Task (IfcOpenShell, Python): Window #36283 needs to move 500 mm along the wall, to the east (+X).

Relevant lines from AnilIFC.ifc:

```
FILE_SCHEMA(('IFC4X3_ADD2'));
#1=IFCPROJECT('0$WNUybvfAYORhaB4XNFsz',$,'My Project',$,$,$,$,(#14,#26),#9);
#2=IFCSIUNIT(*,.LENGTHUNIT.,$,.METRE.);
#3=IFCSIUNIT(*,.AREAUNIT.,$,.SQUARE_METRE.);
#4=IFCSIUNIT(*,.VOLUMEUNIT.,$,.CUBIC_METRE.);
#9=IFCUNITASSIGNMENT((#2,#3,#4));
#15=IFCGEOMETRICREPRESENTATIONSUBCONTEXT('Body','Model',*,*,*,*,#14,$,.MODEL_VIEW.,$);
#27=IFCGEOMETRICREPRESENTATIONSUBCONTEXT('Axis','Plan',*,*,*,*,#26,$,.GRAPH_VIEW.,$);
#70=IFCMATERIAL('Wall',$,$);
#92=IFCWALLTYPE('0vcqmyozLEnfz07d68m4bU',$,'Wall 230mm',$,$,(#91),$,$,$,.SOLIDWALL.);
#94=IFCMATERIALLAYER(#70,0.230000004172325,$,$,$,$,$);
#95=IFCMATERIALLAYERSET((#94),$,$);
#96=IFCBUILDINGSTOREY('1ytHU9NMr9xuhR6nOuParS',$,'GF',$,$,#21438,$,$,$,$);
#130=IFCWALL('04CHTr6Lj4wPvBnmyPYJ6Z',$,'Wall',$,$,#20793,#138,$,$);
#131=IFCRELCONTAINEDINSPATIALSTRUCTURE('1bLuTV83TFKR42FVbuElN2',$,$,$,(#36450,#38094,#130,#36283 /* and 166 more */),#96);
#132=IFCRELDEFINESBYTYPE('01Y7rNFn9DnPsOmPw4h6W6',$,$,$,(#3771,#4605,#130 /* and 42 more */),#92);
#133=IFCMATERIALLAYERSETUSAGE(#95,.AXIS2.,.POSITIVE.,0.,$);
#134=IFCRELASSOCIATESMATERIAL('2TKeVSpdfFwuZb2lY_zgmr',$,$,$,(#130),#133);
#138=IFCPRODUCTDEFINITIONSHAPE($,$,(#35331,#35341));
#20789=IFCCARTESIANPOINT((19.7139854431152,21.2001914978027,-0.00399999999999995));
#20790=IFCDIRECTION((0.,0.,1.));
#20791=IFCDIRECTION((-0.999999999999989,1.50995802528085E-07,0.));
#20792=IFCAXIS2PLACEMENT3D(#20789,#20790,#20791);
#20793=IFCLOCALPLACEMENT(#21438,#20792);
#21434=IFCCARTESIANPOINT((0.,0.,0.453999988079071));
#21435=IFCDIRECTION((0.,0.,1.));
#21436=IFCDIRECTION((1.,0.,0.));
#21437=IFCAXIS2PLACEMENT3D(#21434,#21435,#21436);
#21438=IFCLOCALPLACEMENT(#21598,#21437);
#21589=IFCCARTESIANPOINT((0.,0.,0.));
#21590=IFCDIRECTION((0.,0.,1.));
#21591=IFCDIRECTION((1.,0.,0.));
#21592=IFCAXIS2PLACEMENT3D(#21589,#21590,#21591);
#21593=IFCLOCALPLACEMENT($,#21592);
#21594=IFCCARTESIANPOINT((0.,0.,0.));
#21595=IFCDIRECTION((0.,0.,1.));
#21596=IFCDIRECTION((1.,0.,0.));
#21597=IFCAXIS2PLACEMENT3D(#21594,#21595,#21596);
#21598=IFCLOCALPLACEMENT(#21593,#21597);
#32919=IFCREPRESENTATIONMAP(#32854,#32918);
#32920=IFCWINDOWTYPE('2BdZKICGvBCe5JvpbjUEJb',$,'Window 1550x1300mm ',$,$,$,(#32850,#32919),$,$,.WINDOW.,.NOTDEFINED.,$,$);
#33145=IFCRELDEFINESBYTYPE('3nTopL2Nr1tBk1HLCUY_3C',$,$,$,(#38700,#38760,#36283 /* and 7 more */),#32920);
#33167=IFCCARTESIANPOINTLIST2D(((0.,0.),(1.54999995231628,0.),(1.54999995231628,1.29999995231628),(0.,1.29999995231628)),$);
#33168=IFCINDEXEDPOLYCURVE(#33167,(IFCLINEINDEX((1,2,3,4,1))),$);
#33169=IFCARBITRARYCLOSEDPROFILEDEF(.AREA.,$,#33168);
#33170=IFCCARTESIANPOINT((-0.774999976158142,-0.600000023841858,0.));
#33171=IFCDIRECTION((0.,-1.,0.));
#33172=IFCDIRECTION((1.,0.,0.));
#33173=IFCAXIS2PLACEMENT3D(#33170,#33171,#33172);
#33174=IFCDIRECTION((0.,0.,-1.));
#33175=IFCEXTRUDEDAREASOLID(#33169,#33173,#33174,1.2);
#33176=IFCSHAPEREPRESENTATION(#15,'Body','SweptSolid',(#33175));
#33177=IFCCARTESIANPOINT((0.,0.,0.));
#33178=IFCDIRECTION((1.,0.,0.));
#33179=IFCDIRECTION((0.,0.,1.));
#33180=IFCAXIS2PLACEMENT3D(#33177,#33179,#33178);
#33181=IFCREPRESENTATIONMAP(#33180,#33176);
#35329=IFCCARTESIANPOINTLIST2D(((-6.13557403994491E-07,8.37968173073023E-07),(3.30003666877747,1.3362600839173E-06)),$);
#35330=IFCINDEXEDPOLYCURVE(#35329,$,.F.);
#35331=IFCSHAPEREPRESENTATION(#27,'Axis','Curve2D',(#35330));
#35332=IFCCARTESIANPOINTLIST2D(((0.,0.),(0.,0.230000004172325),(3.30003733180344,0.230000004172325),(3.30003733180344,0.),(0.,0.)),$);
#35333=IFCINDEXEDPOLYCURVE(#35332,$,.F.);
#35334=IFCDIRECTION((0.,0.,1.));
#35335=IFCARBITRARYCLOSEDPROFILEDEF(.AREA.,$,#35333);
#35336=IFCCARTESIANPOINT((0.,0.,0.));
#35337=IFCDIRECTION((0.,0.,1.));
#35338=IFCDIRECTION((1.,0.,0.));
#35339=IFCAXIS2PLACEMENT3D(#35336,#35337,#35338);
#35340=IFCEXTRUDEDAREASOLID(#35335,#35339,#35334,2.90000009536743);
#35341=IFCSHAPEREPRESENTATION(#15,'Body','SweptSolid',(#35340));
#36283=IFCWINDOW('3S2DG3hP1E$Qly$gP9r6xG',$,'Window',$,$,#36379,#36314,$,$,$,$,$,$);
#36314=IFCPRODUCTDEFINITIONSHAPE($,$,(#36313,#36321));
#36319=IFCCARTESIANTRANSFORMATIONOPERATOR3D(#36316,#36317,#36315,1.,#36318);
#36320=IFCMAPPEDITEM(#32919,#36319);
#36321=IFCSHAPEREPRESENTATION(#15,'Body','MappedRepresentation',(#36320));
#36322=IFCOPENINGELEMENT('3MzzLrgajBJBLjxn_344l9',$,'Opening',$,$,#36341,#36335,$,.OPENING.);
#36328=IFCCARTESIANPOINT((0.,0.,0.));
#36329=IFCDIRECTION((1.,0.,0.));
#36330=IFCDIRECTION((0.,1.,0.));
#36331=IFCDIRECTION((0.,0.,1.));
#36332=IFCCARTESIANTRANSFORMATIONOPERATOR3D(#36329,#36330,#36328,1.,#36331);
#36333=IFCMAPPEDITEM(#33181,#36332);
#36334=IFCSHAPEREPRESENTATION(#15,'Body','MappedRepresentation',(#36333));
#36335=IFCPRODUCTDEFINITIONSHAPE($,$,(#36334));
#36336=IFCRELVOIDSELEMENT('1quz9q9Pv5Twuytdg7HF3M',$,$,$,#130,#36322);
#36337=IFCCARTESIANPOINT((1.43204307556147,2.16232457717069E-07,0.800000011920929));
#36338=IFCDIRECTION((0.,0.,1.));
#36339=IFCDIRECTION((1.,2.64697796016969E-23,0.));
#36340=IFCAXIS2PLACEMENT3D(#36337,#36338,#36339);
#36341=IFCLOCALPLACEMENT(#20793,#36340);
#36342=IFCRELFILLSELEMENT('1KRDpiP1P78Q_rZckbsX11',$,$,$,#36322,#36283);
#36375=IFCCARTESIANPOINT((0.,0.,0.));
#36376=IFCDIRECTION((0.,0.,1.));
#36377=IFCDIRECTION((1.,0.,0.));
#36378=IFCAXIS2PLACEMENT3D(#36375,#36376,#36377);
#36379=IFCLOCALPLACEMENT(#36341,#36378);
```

```python
import ifcopenshell
import ifcopenshell.api.geometry
import ifcopenshell.util.placement

model = ifcopenshell.open("AnilIFC.ifc")

window = model.by_guid("3S2DG3hP1E$Qly$gP9r6xG")
opening = window.FillsVoids[0].RelatingOpeningElement
wall = opening.VoidsElements[0].RelatingBuildingElement

wall_matrix = ifcopenshell.util.placement.get_local_placement(wall.ObjectPlacement)
shift = wall_matrix[:3, 0] * -0.5
before = ifcopenshell.util.placement.get_local_placement(window.ObjectPlacement)[:3, 3].copy()

# The window is placed relative to its opening, so it follows when the opening moves.
matrix = ifcopenshell.util.placement.get_local_placement(opening.ObjectPlacement)
matrix[:3, 3] += shift
ifcopenshell.api.geometry.edit_object_placement(
    model, product=opening, matrix=matrix, is_si=False, should_transform_children=True
)

after = ifcopenshell.util.placement.get_local_placement(window.ObjectPlacement)[:3, 3]
print("window moved by", (after - before).round(3) + 0.0)

model.write("AnilIFC_updated.ifc")
```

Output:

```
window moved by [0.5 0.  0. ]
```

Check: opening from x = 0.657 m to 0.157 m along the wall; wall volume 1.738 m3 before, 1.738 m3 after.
